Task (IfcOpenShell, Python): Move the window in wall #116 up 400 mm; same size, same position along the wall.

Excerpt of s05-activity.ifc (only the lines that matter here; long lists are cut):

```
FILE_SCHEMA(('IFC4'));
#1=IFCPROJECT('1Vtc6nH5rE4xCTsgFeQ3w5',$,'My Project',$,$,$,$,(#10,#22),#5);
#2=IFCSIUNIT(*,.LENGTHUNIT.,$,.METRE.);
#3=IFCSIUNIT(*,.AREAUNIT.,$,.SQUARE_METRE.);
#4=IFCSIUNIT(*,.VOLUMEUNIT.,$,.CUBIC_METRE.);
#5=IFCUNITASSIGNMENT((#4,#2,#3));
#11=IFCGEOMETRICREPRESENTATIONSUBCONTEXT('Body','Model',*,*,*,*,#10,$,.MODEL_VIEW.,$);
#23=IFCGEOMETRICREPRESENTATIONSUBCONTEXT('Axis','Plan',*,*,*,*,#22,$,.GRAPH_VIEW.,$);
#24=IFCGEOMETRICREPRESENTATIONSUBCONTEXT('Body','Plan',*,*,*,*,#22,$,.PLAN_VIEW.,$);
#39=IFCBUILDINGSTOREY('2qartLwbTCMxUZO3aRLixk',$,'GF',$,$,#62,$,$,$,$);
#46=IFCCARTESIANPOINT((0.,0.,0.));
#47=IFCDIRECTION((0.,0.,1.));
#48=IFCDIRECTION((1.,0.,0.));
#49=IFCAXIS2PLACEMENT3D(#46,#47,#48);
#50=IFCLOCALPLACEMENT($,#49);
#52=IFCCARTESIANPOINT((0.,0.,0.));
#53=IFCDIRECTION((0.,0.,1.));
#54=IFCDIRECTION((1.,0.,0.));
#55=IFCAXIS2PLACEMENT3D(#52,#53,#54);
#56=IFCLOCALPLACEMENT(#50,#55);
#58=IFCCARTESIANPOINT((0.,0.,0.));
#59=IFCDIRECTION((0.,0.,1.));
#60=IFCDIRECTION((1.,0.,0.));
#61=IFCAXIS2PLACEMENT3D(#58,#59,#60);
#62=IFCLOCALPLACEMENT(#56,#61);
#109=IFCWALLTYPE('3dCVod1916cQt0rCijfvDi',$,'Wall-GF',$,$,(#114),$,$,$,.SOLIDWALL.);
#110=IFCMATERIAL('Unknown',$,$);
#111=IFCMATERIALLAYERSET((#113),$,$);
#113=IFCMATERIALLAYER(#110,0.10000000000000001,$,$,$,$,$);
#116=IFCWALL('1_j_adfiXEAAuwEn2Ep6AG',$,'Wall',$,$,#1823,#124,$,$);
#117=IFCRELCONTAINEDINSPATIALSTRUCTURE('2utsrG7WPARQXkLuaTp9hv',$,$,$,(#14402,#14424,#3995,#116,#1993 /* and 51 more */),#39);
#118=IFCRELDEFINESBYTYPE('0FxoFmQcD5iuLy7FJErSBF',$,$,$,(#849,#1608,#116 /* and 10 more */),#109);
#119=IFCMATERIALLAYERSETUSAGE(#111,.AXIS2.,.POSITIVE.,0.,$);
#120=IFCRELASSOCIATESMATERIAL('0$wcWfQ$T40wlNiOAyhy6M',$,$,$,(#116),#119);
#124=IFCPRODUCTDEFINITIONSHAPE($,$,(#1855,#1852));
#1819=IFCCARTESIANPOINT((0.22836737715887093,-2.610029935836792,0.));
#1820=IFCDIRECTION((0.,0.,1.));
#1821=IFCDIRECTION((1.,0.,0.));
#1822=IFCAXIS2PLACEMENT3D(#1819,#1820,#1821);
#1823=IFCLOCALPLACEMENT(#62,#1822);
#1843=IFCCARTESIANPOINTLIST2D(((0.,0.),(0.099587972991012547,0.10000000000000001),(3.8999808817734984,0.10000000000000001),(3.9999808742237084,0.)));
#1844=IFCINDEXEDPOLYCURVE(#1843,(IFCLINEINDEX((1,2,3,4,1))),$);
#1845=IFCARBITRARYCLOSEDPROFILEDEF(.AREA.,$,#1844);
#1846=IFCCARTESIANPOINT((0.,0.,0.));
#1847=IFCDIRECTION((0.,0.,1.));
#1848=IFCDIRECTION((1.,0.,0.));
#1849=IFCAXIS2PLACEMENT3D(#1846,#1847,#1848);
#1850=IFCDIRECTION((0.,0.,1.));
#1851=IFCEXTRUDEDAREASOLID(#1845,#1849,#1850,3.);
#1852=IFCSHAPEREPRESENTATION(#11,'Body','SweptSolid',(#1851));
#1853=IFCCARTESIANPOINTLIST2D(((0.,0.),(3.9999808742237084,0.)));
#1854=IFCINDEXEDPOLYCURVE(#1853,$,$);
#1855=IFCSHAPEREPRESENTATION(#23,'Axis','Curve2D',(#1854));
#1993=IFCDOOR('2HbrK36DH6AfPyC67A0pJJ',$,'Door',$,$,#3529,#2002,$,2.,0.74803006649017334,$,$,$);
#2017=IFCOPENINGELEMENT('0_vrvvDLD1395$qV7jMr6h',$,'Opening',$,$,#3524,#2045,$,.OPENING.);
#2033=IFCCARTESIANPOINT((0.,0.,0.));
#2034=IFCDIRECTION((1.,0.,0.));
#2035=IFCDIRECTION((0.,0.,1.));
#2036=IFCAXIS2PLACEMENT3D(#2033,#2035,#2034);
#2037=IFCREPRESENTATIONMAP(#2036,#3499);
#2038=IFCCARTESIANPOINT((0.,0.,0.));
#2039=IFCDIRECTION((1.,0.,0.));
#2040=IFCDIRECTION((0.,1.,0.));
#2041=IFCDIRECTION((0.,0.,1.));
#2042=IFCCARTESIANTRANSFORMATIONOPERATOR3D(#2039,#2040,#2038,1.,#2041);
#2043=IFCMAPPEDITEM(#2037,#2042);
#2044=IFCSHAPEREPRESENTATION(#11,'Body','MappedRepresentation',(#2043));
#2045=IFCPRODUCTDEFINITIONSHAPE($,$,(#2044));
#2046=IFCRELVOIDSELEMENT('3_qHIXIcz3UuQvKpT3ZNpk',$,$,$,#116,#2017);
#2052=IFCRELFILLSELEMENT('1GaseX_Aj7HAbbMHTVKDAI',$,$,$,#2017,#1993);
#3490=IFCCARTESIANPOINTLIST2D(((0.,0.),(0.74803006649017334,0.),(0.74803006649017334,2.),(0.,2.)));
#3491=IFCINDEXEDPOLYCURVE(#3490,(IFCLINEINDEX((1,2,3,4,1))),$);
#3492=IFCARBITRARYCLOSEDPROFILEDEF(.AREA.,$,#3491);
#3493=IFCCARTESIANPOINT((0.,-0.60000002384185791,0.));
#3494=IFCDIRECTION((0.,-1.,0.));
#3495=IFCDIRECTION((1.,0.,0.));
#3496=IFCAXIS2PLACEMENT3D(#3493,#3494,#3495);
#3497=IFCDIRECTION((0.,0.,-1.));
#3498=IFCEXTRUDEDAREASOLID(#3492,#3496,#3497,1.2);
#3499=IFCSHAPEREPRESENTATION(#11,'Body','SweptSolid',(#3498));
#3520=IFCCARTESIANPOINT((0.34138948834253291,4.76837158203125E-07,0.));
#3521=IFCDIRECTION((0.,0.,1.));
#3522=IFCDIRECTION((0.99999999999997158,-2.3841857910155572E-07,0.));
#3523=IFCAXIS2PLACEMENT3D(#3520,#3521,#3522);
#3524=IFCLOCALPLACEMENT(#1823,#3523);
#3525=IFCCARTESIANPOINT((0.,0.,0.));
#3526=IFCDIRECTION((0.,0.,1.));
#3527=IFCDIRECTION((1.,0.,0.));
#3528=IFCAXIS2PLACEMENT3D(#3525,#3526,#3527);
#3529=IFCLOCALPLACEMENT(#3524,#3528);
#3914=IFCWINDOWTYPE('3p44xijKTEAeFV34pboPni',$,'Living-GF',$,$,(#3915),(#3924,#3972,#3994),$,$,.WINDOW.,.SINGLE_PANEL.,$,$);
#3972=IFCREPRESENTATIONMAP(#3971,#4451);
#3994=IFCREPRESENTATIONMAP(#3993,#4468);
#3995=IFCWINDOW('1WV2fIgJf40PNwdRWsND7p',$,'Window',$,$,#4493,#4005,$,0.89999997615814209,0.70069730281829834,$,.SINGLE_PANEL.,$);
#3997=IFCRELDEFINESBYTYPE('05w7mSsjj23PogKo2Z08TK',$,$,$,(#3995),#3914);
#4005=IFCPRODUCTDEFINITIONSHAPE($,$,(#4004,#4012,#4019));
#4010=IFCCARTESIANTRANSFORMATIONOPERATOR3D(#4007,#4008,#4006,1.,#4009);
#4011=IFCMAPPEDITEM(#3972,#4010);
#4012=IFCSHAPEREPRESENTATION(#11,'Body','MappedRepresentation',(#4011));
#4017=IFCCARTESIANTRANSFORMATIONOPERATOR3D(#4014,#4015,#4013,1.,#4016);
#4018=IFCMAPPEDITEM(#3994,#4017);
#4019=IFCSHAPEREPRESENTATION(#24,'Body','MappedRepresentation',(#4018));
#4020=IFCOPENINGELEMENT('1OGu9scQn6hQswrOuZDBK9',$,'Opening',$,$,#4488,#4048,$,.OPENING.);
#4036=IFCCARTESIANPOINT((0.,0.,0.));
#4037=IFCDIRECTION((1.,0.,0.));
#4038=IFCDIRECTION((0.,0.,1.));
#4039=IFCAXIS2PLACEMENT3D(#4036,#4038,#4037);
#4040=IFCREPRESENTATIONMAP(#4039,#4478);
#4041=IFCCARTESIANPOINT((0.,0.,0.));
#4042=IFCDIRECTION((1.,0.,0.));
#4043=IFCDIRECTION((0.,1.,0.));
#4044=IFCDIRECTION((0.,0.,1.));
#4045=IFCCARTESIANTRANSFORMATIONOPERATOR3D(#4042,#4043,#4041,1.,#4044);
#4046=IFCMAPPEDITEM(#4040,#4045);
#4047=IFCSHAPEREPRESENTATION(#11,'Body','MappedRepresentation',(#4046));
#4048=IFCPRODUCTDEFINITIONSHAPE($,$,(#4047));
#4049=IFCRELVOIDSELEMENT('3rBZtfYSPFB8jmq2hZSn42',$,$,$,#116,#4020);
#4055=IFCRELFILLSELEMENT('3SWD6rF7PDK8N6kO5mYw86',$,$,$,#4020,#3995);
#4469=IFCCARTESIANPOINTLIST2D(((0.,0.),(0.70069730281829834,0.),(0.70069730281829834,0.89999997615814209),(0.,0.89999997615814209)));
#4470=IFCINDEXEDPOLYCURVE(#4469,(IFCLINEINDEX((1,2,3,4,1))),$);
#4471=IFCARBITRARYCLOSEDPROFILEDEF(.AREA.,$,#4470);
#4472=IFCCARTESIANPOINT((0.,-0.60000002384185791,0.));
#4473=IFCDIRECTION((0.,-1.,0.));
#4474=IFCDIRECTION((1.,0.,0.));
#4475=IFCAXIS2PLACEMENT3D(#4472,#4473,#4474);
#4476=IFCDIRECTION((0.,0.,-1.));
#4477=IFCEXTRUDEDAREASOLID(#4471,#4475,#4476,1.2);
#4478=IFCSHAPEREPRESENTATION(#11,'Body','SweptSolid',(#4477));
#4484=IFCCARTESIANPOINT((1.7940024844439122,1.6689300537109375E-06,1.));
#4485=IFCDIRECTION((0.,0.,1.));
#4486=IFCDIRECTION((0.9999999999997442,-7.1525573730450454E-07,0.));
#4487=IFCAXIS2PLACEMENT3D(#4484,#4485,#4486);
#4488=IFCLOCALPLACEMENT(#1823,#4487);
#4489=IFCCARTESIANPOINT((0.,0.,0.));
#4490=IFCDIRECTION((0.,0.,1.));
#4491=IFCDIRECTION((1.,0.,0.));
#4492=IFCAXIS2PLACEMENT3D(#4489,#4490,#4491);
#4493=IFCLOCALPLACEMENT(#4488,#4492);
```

```python
import numpy as np
import ifcopenshell
import ifcopenshell.api.geometry
import ifcopenshell.util.placement
import ifcopenshell.util.unit

model = ifcopenshell.open("s05-activity.ifc")
unit_scale = ifcopenshell.util.unit.calculate_unit_scale(model)

window = model.by_id(3995)
opening = window.FillsVoids[0].RelatingOpeningElement
dz = 0.4 / unit_scale

shift = np.array([0.0, 0.0, dz])
# The window is placed relative to its opening, so it follows when the opening moves.
matrix = ifcopenshell.util.placement.get_local_placement(opening.ObjectPlacement)
matrix[:3, 3] += shift
ifcopenshell.api.geometry.edit_object_placement(
    model, product=opening, matrix=matrix, is_si=False, should_transform_children=True
)

print(f"moved by {dz * unit_scale:+.3f} m")

model.write("s05-activity_updated.ifc")
```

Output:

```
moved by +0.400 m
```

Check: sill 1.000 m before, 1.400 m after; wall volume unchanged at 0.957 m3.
